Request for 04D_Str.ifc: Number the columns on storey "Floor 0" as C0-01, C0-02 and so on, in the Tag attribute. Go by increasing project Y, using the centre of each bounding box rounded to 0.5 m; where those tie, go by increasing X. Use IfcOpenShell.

First a look at what the model holds.

```python
import ifcopenshell
import ifcopenshell.util.element
import ifcopenshell.util.placement

model = ifcopenshell.open("04D_Str.ifc")
print(model.schema)
storey = next(s for s in model.by_type("IfcBuildingStorey") if s.Name == "Floor 0")
columns = [e for e in ifcopenshell.util.element.get_decomposition(storey) if e.is_a("IfcColumn")]
for e in sorted(columns, key=lambda e: e.id()):
    origin = ifcopenshell.util.placement.get_local_placement(e.ObjectPlacement)[:3, 3]
    print(e.id(), e.Tag, e.Name, origin.round(2) + 0.0, sep=" | ")
```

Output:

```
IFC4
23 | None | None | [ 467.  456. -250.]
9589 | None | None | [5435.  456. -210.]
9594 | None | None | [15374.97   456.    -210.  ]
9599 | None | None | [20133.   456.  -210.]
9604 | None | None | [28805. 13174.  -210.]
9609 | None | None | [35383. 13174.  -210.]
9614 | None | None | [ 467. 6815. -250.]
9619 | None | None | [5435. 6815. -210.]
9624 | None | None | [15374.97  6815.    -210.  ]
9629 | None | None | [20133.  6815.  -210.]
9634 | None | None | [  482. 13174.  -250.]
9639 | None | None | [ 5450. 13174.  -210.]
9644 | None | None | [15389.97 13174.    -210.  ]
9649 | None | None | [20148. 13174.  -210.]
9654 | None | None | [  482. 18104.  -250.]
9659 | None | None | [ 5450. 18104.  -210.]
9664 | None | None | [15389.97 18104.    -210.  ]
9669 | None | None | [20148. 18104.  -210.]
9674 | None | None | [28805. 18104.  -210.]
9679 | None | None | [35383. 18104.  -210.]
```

```python
import ifcopenshell
import ifcopenshell.geom
import ifcopenshell.util.element
import ifcopenshell.util.shape

model = ifcopenshell.open("04D_Str.ifc")
settings = ifcopenshell.geom.settings()
settings.set("use-world-coords", True)


def centre(element):
    shape = ifcopenshell.geom.create_shape(settings, element)
    return ifcopenshell.util.shape.get_bbox_centroid(shape.geometry)


storey = next(s for s in model.by_type("IfcBuildingStorey") if s.Name == "Floor 0")
columns = [e for e in ifcopenshell.util.element.get_decomposition(storey) if e.is_a("IfcColumn")]

# Insertion points can sit at a corner or the storey origin, so sort by the geometry (in metres).
centres = {e: centre(e) for e in columns}
columns.sort(key=lambda e: (round(centres[e][1] / 0.5), centres[e][0]))

for i, e in enumerate(columns, start=1):
    number = f"C0-{i:02d}"
    e.Tag = number
    print(e.id(), number)

model.write("04D_Str_rev.ifc")
```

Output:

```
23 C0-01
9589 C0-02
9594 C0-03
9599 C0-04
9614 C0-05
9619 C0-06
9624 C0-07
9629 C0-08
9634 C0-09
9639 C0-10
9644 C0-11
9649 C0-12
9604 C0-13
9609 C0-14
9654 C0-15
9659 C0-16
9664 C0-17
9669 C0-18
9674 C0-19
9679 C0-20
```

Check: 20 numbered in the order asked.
